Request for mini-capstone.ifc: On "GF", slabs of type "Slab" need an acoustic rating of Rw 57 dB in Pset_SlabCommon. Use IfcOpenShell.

First a look at what the model holds.

```python
import ifcopenshell
import ifcopenshell.util.element

model = ifcopenshell.open("mini-capstone.ifc")
print(model.schema)
storey = next(s for s in model.by_type("IfcBuildingStorey") if s.Name == "GF")
slabs = [e for e in ifcopenshell.util.element.get_decomposition(storey) if e.is_a("IfcSlab")]
seen = {}
for e in slabs:
    element_type = ifcopenshell.util.element.get_type(e)
    key = (element_type.Name if element_type != e and element_type else None, ifcopenshell.util.element.get_pset(e, "Pset_SlabCommon", "AcousticRating"))
    seen[key] = seen.get(key, 0) + 1
for (name, value), count in sorted(seen.items(), key=str):
    print(count, "x", name, "|", value)
```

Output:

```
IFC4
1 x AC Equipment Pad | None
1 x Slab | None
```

```python
import ifcopenshell
import ifcopenshell.api.pset
import ifcopenshell.util.element

model = ifcopenshell.open("mini-capstone.ifc")

storey = next(s for s in model.by_type("IfcBuildingStorey") if s.Name == "GF")
slabs = [e for e in ifcopenshell.util.element.get_decomposition(storey) if e.is_a("IfcSlab")]

count = 0
for e in slabs:
    element_type = ifcopenshell.util.element.get_type(e)
    if element_type in (None, e) or element_type.Name != "Slab":
        continue
    # add_pset returns the element's existing set when there is one.
    pset = ifcopenshell.api.pset.add_pset(model, product=e, name="Pset_SlabCommon")
    ifcopenshell.api.pset.edit_pset(model, pset=pset, properties={"AcousticRating": "Rw 57 dB"})
    count += 1

print(count, "slabs updated")

model.write("mini-capstone-out.ifc")
```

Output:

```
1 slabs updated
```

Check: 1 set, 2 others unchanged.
